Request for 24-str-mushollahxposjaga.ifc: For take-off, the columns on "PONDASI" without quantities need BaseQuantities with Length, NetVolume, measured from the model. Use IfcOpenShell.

First a look at what the model holds.

```python
import ifcopenshell
import ifcopenshell.util.element
import ifcopenshell.util.unit

model = ifcopenshell.open("24-str-mushollahxposjaga.ifc")
print(model.schema)
for unit_type in ("LENGTHUNIT", "AREAUNIT", "VOLUMEUNIT"):
    print(unit_type, ifcopenshell.util.unit.calculate_unit_scale(model, unit_type))
storey = next(s for s in model.by_type("IfcBuildingStorey") if s.Name == "PONDASI")
columns = [e for e in ifcopenshell.util.element.get_decomposition(storey) if e.is_a("IfcColumn")]
for e in sorted(columns, key=lambda e: e.id()):
    print(e.id(), e.is_a(), e.Name, list(ifcopenshell.util.element.get_psets(e, qtos_only=True)), sep=" | ")
```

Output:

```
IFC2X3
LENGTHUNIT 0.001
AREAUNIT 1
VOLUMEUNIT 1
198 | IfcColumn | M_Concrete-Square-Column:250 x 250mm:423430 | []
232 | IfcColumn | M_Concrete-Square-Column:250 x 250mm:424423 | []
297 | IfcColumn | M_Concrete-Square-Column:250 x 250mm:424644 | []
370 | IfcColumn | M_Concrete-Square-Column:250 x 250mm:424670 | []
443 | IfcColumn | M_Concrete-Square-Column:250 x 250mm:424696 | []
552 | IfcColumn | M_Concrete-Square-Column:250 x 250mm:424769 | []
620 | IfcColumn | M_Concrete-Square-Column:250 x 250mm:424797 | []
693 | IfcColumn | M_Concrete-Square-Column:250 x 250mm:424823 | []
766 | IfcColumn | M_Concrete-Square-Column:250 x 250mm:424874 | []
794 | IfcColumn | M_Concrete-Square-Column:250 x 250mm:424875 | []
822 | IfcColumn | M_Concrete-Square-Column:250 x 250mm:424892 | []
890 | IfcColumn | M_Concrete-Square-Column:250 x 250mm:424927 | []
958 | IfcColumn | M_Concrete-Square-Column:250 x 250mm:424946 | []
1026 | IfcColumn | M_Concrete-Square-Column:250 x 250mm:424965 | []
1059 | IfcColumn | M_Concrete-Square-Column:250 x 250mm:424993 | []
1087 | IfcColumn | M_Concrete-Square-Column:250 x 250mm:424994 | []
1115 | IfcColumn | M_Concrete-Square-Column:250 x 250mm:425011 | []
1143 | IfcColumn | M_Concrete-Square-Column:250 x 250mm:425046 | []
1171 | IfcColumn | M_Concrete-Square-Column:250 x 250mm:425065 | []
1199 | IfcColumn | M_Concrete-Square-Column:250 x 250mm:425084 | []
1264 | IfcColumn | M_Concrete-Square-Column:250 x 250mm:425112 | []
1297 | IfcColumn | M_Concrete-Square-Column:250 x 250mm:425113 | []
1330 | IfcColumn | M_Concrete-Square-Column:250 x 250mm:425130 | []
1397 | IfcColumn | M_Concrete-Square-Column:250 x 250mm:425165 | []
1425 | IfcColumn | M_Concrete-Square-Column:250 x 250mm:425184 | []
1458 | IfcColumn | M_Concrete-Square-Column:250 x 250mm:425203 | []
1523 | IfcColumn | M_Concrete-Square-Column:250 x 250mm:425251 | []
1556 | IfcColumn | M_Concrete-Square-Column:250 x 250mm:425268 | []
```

```python
import ifcopenshell
import ifcopenshell.api.pset
import ifcopenshell.geom
import ifcopenshell.util.element
import ifcopenshell.util.shape
import ifcopenshell.util.unit

model = ifcopenshell.open("24-str-mushollahxposjaga.ifc")
unit_scale = ifcopenshell.util.unit.calculate_unit_scale(model)
volume_scale = ifcopenshell.util.unit.calculate_unit_scale(model, "VOLUMEUNIT")
settings = ifcopenshell.geom.settings()

storey = next(s for s in model.by_type("IfcBuildingStorey") if s.Name == "PONDASI")
columns = [e for e in ifcopenshell.util.element.get_decomposition(storey) if e.is_a("IfcColumn")]

for e in sorted(columns, key=lambda e: e.id()):
    if ifcopenshell.util.element.get_psets(e, qtos_only=True, should_inherit=False):
        continue
    # Geometry comes back in metres, in the element's own axes.
    shape = ifcopenshell.geom.create_shape(settings, e)
    values = {
        "Length": ifcopenshell.util.shape.get_z(shape.geometry) / unit_scale,
        "NetVolume": ifcopenshell.util.shape.get_volume(shape.geometry) / volume_scale,
    }
    qto = ifcopenshell.api.pset.add_qto(model, product=e, name="BaseQuantities")
    ifcopenshell.api.pset.edit_qto(model, qto=qto, properties=values)
    print(e.id(), {k: round(v, 3) for k, v in values.items()})

model.write("24-str-mushollahxposjaga_rev.ifc")
```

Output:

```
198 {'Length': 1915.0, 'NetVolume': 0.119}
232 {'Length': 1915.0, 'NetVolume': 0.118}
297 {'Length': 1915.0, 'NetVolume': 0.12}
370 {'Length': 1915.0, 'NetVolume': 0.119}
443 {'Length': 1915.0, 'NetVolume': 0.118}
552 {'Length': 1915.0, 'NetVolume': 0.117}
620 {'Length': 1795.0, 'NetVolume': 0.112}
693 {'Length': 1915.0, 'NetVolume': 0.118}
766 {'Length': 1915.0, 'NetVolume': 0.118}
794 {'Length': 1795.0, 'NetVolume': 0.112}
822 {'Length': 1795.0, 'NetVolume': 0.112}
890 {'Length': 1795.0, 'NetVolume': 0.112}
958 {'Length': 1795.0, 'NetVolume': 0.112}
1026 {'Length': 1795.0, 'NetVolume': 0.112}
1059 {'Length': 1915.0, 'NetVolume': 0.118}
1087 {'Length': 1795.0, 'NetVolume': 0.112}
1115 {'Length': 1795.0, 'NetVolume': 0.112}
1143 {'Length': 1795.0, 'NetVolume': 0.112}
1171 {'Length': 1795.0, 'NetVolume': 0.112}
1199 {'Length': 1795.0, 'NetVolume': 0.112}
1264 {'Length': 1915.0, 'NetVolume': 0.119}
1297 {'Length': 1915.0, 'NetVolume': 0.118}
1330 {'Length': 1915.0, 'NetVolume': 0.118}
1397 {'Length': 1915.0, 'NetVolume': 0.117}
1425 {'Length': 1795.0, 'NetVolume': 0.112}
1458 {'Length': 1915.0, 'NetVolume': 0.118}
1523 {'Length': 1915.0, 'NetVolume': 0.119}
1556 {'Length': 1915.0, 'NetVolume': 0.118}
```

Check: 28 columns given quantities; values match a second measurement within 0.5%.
